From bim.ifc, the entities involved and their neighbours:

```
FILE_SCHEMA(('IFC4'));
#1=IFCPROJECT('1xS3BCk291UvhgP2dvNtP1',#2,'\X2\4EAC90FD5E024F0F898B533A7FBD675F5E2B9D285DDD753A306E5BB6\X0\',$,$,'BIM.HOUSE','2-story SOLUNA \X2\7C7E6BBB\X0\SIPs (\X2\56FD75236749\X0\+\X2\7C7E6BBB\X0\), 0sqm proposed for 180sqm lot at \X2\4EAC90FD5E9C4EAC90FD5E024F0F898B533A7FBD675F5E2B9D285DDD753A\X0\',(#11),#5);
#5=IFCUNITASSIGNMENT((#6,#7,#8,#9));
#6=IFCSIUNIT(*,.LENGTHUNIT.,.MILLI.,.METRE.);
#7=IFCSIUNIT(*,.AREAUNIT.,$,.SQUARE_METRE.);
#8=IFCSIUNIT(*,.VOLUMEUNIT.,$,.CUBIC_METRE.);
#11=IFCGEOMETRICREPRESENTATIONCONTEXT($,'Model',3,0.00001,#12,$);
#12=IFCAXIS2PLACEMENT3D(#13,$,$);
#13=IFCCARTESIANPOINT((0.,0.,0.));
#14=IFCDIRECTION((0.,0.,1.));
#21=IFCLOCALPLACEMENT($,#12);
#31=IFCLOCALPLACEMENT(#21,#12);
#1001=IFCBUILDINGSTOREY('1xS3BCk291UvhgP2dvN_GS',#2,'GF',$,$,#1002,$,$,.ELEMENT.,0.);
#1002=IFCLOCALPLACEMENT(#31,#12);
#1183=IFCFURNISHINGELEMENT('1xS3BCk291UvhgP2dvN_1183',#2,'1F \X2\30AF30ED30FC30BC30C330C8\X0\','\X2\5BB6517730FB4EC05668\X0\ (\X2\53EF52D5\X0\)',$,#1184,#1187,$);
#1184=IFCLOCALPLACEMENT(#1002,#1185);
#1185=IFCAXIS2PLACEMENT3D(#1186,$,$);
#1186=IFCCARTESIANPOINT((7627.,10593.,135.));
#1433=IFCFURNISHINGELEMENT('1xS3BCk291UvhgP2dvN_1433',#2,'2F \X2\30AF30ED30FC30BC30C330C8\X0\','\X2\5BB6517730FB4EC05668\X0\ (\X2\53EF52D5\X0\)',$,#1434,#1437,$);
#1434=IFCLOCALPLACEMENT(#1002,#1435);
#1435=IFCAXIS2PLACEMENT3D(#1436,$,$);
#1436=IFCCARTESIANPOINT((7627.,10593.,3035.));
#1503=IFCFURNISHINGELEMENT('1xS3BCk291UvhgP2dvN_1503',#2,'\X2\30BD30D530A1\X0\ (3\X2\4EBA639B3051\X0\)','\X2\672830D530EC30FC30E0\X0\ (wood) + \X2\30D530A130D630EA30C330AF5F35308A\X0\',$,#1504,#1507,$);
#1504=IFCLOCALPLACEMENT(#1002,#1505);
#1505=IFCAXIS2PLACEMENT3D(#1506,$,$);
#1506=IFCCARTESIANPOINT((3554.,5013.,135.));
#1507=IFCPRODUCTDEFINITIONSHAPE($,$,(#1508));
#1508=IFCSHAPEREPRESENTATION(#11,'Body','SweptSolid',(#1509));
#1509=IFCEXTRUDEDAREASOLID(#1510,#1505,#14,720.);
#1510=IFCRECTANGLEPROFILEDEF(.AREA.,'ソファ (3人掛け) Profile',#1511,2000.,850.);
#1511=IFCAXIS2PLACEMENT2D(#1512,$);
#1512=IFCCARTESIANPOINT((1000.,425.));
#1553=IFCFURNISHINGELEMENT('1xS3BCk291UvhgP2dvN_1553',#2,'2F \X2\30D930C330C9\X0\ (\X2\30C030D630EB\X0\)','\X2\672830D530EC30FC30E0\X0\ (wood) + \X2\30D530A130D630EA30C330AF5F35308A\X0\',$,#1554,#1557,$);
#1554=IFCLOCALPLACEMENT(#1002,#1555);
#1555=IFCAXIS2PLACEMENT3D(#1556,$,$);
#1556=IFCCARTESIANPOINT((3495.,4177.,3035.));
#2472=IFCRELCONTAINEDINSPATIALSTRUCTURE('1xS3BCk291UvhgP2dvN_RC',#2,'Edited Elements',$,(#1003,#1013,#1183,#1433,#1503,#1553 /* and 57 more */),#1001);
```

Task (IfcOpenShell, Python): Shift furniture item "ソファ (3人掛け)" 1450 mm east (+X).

```python
import ifcopenshell
import ifcopenshell.api.geometry
import ifcopenshell.util.placement
import ifcopenshell.util.unit

model = ifcopenshell.open("bim.ifc")
unit_scale = ifcopenshell.util.unit.calculate_unit_scale(model)

item = model.by_id(1503)
matrix = ifcopenshell.util.placement.get_local_placement(item.ObjectPlacement)
matrix[0, 3] += 1.45 / unit_scale
ifcopenshell.api.geometry.edit_object_placement(model, product=item, matrix=matrix, is_si=False)

print(ifcopenshell.util.placement.get_local_placement(item.ObjectPlacement).round(3) + 0.0)

model.write("bim_v2.ifc")
```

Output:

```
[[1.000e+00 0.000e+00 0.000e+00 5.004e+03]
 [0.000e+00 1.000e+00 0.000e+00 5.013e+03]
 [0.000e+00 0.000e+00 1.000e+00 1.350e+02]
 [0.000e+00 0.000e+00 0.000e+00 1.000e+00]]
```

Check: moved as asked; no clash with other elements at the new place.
